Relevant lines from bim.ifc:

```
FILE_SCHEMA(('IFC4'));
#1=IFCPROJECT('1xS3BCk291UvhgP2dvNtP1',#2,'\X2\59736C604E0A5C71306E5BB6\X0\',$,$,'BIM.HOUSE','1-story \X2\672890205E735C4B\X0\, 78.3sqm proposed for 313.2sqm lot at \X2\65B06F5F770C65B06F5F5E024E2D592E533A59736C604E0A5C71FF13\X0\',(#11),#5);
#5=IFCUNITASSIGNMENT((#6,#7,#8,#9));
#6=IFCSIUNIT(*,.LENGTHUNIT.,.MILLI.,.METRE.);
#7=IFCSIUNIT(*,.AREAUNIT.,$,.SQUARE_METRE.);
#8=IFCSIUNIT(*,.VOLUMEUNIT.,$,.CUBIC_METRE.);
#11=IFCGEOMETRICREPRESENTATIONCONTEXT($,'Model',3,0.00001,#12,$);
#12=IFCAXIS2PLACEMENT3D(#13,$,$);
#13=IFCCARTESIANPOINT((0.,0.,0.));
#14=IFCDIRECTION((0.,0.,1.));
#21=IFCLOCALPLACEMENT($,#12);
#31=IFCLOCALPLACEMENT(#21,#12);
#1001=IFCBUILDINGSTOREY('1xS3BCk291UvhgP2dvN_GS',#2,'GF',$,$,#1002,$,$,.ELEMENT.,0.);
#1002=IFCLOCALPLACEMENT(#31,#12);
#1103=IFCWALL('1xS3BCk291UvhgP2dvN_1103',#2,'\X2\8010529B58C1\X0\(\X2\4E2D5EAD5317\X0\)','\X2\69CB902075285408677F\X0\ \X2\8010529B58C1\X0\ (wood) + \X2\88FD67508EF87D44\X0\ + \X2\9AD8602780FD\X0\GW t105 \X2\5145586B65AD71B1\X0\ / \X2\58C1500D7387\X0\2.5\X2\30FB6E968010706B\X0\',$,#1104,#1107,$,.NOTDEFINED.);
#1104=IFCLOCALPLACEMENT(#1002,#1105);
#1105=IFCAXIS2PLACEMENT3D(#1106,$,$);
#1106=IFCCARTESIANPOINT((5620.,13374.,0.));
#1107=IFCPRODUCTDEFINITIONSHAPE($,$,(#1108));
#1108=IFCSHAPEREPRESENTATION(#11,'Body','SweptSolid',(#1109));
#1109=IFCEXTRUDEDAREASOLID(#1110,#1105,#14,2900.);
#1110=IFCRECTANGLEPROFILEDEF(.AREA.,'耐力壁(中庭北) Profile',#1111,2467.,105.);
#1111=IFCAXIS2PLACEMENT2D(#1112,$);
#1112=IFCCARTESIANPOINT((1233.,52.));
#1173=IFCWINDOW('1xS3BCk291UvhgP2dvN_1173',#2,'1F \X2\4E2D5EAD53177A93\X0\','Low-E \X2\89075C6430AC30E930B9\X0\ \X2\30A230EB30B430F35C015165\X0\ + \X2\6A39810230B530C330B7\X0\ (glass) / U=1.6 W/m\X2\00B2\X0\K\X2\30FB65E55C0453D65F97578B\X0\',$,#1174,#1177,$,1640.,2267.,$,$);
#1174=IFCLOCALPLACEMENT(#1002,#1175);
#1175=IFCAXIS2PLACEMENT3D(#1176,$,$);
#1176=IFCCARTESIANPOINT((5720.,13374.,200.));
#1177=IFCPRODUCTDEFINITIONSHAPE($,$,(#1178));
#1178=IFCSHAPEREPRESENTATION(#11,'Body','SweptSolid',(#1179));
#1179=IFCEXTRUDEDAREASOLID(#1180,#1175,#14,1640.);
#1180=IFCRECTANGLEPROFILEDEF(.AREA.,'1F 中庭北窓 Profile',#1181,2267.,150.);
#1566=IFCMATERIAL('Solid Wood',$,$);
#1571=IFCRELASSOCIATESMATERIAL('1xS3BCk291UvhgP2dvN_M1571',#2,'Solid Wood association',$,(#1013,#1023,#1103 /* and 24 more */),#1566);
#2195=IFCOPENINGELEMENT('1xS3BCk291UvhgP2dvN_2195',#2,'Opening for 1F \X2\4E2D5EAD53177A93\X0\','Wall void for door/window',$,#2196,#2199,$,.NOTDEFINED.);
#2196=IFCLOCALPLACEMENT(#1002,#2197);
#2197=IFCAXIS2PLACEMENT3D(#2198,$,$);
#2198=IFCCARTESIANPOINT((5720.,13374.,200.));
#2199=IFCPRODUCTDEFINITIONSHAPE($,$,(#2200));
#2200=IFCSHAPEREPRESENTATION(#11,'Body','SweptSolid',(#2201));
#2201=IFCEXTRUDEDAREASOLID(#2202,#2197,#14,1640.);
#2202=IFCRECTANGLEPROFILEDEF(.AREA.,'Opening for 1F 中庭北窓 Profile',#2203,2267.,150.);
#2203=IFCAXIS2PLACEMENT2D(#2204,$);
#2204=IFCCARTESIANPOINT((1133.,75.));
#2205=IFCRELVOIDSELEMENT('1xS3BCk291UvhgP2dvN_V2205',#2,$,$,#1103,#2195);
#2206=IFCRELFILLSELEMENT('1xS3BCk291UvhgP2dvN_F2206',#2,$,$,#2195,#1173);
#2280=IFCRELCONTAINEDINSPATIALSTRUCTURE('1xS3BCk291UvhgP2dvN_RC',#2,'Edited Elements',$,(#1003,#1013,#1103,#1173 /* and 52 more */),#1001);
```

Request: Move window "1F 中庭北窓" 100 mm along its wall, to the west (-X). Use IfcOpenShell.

```python
import ifcopenshell
import ifcopenshell.api.geometry
import ifcopenshell.util.placement
import ifcopenshell.util.unit

model = ifcopenshell.open("bim.ifc")
unit_scale = ifcopenshell.util.unit.calculate_unit_scale(model)

window = model.by_guid("1xS3BCk291UvhgP2dvN_1173")
opening = window.FillsVoids[0].RelatingOpeningElement
wall = opening.VoidsElements[0].RelatingBuildingElement

wall_matrix = ifcopenshell.util.placement.get_local_placement(wall.ObjectPlacement)
shift = wall_matrix[:3, 0] * -0.1 / unit_scale
before = ifcopenshell.util.placement.get_local_placement(window.ObjectPlacement)[:3, 3].copy()

# The window is not placed relative to its opening, so move both.
for product in (opening, window):
    matrix = ifcopenshell.util.placement.get_local_placement(product.ObjectPlacement)
    matrix[:3, 3] += shift
    ifcopenshell.api.geometry.edit_object_placement(model, product=product, matrix=matrix, is_si=False)

after = ifcopenshell.util.placement.get_local_placement(window.ObjectPlacement)[:3, 3]
print("window moved by", (after - before).round(3) + 0.0)

model.write("bim_v2.ifc")
```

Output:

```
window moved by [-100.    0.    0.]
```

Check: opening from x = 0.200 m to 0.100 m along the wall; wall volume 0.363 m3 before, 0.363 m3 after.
